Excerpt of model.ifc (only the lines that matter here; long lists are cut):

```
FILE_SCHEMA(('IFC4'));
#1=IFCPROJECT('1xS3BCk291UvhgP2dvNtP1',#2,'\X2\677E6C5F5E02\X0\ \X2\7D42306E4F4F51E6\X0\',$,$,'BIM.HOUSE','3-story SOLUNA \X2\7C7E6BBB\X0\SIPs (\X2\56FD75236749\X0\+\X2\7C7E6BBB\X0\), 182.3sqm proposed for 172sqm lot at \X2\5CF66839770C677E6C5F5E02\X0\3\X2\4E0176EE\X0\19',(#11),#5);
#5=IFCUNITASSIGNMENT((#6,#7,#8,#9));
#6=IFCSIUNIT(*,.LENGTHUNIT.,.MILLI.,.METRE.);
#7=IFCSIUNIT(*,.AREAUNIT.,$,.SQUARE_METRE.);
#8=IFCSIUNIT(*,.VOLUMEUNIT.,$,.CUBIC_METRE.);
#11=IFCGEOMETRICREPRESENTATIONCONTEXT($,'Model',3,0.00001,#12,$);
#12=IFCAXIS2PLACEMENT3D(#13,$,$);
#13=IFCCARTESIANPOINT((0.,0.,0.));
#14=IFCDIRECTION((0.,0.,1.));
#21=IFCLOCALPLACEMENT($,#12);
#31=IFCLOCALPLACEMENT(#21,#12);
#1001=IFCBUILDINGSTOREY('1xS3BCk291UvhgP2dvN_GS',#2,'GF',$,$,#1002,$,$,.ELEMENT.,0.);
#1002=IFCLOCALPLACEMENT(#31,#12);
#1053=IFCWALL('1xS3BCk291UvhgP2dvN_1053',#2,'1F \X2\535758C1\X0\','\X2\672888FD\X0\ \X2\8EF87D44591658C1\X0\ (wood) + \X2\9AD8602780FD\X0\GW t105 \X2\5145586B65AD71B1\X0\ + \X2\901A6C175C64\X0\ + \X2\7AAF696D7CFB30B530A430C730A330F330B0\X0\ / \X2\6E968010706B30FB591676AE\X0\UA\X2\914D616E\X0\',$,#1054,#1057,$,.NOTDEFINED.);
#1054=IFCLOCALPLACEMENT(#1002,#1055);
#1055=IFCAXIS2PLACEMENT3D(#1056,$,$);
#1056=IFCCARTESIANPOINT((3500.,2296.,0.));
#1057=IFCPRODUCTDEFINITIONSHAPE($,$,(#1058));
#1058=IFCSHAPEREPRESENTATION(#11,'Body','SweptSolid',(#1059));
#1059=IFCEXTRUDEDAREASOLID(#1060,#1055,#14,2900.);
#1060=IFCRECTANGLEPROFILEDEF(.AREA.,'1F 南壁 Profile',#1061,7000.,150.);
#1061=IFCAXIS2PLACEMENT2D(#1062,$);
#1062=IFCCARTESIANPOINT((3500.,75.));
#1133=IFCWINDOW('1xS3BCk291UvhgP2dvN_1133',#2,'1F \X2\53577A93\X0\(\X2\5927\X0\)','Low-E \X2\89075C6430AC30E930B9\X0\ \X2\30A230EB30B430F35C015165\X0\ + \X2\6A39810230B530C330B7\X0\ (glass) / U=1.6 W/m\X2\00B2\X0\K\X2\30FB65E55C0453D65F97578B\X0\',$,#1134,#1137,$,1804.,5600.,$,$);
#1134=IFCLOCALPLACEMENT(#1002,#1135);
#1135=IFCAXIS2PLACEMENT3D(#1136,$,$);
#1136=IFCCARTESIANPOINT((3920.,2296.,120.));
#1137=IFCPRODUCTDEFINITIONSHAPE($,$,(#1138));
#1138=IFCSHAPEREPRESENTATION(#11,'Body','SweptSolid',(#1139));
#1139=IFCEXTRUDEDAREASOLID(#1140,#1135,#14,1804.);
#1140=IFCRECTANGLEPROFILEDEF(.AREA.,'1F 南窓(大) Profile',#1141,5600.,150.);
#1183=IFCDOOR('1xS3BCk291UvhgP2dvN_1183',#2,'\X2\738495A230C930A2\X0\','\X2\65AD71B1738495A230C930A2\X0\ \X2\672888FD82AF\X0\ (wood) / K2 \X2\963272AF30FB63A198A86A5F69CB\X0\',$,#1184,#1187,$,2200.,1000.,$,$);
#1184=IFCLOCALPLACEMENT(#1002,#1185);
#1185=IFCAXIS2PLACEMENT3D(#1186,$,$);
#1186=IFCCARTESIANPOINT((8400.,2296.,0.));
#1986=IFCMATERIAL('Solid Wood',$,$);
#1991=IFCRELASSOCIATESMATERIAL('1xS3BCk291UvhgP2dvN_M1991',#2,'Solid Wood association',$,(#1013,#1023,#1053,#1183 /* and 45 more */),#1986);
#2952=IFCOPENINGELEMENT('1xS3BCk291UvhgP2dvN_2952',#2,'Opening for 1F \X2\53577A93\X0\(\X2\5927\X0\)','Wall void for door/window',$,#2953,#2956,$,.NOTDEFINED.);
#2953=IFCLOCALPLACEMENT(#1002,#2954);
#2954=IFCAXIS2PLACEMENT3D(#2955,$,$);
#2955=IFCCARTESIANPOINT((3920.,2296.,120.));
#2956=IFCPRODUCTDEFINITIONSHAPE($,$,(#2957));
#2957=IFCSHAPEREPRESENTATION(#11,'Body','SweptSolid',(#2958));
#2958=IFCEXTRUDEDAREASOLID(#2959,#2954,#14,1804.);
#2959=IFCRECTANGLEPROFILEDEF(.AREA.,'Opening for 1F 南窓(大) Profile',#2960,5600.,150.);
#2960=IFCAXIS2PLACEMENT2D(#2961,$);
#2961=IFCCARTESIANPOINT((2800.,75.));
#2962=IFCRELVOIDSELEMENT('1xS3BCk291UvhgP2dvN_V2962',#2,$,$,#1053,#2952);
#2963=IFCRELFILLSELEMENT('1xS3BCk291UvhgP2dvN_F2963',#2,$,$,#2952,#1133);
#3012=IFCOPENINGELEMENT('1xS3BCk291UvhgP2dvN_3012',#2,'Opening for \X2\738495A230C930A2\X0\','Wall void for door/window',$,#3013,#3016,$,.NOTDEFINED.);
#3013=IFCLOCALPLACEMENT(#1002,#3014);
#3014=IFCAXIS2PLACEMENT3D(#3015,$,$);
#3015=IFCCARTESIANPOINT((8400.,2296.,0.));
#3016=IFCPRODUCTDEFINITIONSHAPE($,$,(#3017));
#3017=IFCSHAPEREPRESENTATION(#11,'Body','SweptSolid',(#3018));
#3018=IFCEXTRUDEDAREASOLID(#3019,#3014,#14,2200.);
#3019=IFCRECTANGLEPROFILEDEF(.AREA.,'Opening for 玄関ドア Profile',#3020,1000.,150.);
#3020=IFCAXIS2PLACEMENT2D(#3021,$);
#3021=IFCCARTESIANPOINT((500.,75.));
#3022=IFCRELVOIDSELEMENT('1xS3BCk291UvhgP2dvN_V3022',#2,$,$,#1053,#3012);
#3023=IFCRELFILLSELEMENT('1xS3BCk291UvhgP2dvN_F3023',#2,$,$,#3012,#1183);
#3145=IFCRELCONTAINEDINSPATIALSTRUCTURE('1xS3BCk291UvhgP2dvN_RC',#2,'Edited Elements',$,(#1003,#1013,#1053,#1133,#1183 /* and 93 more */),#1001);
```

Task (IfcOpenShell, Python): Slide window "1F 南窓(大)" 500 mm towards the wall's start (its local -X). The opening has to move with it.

```python
import ifcopenshell
import ifcopenshell.api.geometry
import ifcopenshell.util.placement
import ifcopenshell.util.unit

model = ifcopenshell.open("model.ifc")
unit_scale = ifcopenshell.util.unit.calculate_unit_scale(model)

window = model.by_guid("1xS3BCk291UvhgP2dvN_1133")
opening = window.FillsVoids[0].RelatingOpeningElement
wall = opening.VoidsElements[0].RelatingBuildingElement

wall_matrix = ifcopenshell.util.placement.get_local_placement(wall.ObjectPlacement)
shift = wall_matrix[:3, 0] * -0.5 / unit_scale
before = ifcopenshell.util.placement.get_local_placement(window.ObjectPlacement)[:3, 3].copy()

# The window is not placed relative to its opening, so move both.
for product in (opening, window):
    matrix = ifcopenshell.util.placement.get_local_placement(product.ObjectPlacement)
    matrix[:3, 3] += shift
    ifcopenshell.api.geometry.edit_object_placement(model, product=product, matrix=matrix, is_si=False)

after = ifcopenshell.util.placement.get_local_placement(window.ObjectPlacement)[:3, 3]
print("window moved by", (after - before).round(3) + 0.0)

model.write("model_edited.ifc")
```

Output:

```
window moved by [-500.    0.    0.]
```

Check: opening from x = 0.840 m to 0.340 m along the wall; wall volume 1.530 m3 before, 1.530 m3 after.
